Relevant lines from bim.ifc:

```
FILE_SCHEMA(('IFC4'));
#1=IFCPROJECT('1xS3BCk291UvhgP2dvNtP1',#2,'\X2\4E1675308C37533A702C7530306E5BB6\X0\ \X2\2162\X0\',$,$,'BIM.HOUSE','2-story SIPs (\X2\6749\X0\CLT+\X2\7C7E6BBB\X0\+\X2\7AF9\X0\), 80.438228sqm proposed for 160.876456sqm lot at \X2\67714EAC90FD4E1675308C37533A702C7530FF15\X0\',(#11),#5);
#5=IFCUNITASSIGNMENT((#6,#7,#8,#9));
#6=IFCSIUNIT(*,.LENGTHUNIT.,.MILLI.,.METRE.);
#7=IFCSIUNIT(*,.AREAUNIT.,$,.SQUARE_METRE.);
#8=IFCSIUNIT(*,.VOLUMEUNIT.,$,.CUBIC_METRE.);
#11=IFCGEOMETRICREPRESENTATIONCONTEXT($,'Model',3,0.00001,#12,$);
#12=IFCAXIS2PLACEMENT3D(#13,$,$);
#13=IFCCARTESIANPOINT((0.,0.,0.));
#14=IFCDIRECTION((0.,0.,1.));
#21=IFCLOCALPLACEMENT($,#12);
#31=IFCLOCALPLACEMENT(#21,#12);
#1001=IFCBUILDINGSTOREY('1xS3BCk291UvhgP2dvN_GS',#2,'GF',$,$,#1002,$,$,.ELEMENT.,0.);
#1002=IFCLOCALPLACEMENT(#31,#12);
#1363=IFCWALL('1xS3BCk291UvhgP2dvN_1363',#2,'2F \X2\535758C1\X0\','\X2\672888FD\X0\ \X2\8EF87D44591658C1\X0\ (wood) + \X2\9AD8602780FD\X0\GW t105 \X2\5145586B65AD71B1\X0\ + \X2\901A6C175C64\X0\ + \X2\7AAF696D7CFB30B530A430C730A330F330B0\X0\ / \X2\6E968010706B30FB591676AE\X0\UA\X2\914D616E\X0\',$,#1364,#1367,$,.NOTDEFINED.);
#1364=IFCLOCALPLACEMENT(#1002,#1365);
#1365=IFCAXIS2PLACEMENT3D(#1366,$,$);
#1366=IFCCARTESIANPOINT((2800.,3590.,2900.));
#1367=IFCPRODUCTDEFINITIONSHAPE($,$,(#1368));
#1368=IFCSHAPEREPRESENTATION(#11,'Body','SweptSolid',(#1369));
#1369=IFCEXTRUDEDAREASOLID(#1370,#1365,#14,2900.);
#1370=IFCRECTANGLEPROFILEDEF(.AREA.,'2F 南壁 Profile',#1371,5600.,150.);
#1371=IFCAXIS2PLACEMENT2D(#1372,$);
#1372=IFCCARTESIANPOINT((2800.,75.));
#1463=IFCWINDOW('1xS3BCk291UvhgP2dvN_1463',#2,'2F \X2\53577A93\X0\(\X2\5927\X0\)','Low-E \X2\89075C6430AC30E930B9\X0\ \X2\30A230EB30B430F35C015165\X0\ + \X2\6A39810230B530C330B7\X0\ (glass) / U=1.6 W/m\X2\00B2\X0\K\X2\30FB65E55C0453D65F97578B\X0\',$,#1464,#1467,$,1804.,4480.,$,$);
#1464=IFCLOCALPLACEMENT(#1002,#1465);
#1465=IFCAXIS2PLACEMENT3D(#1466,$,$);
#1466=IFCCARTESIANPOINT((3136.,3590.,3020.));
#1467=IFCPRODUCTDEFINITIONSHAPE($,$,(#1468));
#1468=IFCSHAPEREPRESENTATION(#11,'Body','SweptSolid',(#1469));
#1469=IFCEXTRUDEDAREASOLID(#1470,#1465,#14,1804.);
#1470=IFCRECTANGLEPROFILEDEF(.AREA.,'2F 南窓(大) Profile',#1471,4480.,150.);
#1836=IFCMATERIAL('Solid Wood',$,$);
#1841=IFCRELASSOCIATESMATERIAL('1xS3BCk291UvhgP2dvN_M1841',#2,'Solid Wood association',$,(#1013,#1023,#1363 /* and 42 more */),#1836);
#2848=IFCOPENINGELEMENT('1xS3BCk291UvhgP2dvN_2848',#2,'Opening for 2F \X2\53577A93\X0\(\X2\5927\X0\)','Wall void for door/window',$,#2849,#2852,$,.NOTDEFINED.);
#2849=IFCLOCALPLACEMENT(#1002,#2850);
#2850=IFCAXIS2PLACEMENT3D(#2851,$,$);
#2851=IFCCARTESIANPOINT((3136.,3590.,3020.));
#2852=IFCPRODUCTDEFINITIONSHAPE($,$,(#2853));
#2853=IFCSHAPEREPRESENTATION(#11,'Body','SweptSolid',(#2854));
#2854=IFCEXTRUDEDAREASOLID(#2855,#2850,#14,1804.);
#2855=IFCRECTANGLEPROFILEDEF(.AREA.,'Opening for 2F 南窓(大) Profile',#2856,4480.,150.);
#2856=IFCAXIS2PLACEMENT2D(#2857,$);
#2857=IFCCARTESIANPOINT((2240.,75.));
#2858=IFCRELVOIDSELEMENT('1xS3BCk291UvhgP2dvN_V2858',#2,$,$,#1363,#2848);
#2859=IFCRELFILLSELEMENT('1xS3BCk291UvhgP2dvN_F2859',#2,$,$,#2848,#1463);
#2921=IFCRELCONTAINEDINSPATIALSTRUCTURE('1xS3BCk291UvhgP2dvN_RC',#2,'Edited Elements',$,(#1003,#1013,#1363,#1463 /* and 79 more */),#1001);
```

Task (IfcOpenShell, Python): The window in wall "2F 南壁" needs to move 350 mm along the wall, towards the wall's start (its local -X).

```python
import ifcopenshell
import ifcopenshell.api.geometry
import ifcopenshell.util.placement
import ifcopenshell.util.unit

model = ifcopenshell.open("bim.ifc")
unit_scale = ifcopenshell.util.unit.calculate_unit_scale(model)

window = model.by_id(1463)
opening = window.FillsVoids[0].RelatingOpeningElement
wall = opening.VoidsElements[0].RelatingBuildingElement

wall_matrix = ifcopenshell.util.placement.get_local_placement(wall.ObjectPlacement)
shift = wall_matrix[:3, 0] * -0.35 / unit_scale
before = ifcopenshell.util.placement.get_local_placement(window.ObjectPlacement)[:3, 3].copy()

# The window is not placed relative to its opening, so move both.
for product in (opening, window):
    matrix = ifcopenshell.util.placement.get_local_placement(product.ObjectPlacement)
    matrix[:3, 3] += shift
    ifcopenshell.api.geometry.edit_object_placement(model, product=product, matrix=matrix, is_si=False)

after = ifcopenshell.util.placement.get_local_placement(window.ObjectPlacement)[:3, 3]
print("window moved by", (after - before).round(3) + 0.0)

model.write("bim_updated.ifc")
```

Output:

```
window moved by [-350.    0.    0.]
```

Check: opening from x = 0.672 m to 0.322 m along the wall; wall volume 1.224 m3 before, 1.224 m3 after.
